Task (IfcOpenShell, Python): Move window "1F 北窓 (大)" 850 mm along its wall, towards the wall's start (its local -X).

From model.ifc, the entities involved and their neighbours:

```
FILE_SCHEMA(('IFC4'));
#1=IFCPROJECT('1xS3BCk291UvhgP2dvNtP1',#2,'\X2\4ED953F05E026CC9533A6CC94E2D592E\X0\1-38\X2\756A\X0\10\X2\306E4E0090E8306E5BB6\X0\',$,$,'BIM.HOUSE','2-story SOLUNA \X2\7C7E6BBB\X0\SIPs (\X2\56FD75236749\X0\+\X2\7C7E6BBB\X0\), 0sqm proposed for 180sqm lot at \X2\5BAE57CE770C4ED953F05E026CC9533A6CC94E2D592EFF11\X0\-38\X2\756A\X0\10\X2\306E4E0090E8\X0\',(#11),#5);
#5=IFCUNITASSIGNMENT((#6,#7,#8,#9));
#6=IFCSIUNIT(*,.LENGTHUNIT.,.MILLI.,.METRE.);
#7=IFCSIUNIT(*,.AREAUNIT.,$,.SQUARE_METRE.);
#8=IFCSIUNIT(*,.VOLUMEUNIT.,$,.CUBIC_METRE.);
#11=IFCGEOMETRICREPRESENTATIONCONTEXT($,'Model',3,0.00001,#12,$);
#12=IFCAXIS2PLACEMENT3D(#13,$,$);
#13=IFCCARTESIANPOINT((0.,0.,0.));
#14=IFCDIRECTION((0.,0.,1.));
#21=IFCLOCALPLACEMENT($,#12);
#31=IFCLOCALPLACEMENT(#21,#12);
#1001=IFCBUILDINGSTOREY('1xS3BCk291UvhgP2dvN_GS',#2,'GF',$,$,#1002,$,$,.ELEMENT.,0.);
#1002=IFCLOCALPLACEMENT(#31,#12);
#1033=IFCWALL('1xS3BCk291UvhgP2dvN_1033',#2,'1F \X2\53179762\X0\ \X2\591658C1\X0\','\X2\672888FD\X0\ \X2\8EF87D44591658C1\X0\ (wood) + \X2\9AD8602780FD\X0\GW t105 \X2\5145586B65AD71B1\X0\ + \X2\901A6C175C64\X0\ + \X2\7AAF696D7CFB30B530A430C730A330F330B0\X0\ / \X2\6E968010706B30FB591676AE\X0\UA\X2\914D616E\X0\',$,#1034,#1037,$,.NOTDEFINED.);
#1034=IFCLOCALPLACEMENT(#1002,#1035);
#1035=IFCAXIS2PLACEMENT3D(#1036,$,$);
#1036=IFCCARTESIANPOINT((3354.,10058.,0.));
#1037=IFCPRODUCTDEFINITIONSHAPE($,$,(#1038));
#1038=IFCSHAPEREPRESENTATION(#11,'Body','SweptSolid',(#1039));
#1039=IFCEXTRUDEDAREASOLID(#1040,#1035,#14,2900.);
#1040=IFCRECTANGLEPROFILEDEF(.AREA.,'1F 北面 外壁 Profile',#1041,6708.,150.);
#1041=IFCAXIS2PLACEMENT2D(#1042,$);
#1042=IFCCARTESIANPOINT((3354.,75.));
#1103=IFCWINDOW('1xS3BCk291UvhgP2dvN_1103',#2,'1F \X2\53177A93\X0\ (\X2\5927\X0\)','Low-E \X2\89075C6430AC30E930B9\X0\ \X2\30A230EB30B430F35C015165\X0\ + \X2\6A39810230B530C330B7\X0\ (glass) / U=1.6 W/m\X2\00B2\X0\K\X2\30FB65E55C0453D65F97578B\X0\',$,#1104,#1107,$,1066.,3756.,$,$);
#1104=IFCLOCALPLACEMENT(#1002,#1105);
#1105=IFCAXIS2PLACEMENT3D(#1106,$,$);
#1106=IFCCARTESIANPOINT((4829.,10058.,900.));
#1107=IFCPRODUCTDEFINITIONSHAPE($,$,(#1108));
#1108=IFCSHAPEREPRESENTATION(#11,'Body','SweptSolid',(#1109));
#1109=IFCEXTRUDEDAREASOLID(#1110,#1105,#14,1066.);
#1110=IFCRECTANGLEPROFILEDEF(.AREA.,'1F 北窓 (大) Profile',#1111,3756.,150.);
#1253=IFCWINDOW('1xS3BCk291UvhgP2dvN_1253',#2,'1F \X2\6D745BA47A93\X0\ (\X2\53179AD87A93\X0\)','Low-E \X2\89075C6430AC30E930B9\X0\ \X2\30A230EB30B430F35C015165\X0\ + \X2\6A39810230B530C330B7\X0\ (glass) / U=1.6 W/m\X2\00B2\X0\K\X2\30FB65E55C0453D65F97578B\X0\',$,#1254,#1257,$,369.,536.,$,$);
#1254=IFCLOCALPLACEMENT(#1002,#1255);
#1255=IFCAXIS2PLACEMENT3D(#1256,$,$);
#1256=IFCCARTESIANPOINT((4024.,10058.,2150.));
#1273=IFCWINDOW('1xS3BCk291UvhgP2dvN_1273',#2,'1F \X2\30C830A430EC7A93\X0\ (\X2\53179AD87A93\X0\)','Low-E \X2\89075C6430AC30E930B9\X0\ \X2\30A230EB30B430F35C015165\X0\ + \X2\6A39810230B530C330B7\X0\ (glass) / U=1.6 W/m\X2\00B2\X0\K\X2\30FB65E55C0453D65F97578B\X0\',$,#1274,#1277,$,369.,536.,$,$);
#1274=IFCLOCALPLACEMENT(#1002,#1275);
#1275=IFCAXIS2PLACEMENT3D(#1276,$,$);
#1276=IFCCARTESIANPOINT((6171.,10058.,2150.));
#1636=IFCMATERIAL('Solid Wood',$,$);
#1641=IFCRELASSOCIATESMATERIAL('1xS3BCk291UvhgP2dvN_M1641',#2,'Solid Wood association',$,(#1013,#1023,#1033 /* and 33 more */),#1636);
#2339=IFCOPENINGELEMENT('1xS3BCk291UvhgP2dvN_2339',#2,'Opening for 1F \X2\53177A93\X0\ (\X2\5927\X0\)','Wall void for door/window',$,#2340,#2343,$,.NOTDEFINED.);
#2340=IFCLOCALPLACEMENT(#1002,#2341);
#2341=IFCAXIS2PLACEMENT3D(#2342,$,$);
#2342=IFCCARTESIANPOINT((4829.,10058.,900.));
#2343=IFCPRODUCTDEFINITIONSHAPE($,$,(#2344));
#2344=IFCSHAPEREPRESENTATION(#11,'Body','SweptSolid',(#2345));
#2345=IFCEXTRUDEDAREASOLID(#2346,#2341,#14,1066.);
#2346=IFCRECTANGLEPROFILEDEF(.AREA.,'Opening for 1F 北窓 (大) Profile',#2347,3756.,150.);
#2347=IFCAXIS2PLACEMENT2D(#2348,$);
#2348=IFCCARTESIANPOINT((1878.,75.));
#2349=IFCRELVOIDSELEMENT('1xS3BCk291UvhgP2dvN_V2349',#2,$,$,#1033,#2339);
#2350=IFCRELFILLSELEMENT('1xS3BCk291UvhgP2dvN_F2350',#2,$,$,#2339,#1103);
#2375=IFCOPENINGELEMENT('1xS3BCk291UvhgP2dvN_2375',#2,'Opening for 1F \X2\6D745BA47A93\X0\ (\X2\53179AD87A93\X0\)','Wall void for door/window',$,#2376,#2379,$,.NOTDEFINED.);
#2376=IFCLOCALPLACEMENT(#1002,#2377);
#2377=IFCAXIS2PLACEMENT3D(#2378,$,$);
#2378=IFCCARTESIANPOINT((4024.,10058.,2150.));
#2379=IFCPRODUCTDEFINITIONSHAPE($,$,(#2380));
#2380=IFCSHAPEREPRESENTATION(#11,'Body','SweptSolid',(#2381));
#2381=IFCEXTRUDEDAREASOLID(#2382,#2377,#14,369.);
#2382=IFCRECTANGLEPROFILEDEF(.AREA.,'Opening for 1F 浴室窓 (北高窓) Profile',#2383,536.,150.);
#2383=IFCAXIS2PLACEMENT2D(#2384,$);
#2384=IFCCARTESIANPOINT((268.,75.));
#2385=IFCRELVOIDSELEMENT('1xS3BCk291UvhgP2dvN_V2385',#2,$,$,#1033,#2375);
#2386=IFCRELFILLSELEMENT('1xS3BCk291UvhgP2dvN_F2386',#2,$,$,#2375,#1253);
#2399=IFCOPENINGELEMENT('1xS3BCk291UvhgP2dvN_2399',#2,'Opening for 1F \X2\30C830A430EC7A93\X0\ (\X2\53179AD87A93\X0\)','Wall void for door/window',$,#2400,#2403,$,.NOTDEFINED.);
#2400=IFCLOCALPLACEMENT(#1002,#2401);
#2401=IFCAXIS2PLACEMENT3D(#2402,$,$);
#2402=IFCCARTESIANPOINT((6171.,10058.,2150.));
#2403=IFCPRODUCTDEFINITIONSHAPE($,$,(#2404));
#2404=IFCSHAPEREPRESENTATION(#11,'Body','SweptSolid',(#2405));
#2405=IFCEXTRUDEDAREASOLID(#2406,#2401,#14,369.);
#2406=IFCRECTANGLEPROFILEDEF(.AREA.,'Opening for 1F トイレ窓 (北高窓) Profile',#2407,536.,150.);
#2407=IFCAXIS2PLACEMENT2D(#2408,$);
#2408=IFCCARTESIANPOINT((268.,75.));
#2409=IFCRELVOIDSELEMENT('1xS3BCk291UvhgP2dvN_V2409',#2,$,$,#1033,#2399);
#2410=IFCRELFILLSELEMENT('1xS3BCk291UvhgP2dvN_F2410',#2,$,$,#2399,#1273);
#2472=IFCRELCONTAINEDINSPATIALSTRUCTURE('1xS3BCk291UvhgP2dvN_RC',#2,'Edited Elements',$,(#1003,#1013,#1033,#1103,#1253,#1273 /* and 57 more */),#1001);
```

```python
import ifcopenshell
import ifcopenshell.api.geometry
import ifcopenshell.util.placement
import ifcopenshell.util.unit

model = ifcopenshell.open("model.ifc")
unit_scale = ifcopenshell.util.unit.calculate_unit_scale(model)

window = model.by_id(1103)
opening = window.FillsVoids[0].RelatingOpeningElement
wall = opening.VoidsElements[0].RelatingBuildingElement

wall_matrix = ifcopenshell.util.placement.get_local_placement(wall.ObjectPlacement)
shift = wall_matrix[:3, 0] * -0.85 / unit_scale
before = ifcopenshell.util.placement.get_local_placement(window.ObjectPlacement)[:3, 3].copy()

# The window is not placed relative to its opening, so move both.
for product in (opening, window):
    matrix = ifcopenshell.util.placement.get_local_placement(product.ObjectPlacement)
    matrix[:3, 3] += shift
    ifcopenshell.api.geometry.edit_object_placement(model, product=product, matrix=matrix, is_si=False)

after = ifcopenshell.util.placement.get_local_placement(window.ObjectPlacement)[:3, 3]
print("window moved by", (after - before).round(3) + 0.0)

model.write("model_edited.ifc")
```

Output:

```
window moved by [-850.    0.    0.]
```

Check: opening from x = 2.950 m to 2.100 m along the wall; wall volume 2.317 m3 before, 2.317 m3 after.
